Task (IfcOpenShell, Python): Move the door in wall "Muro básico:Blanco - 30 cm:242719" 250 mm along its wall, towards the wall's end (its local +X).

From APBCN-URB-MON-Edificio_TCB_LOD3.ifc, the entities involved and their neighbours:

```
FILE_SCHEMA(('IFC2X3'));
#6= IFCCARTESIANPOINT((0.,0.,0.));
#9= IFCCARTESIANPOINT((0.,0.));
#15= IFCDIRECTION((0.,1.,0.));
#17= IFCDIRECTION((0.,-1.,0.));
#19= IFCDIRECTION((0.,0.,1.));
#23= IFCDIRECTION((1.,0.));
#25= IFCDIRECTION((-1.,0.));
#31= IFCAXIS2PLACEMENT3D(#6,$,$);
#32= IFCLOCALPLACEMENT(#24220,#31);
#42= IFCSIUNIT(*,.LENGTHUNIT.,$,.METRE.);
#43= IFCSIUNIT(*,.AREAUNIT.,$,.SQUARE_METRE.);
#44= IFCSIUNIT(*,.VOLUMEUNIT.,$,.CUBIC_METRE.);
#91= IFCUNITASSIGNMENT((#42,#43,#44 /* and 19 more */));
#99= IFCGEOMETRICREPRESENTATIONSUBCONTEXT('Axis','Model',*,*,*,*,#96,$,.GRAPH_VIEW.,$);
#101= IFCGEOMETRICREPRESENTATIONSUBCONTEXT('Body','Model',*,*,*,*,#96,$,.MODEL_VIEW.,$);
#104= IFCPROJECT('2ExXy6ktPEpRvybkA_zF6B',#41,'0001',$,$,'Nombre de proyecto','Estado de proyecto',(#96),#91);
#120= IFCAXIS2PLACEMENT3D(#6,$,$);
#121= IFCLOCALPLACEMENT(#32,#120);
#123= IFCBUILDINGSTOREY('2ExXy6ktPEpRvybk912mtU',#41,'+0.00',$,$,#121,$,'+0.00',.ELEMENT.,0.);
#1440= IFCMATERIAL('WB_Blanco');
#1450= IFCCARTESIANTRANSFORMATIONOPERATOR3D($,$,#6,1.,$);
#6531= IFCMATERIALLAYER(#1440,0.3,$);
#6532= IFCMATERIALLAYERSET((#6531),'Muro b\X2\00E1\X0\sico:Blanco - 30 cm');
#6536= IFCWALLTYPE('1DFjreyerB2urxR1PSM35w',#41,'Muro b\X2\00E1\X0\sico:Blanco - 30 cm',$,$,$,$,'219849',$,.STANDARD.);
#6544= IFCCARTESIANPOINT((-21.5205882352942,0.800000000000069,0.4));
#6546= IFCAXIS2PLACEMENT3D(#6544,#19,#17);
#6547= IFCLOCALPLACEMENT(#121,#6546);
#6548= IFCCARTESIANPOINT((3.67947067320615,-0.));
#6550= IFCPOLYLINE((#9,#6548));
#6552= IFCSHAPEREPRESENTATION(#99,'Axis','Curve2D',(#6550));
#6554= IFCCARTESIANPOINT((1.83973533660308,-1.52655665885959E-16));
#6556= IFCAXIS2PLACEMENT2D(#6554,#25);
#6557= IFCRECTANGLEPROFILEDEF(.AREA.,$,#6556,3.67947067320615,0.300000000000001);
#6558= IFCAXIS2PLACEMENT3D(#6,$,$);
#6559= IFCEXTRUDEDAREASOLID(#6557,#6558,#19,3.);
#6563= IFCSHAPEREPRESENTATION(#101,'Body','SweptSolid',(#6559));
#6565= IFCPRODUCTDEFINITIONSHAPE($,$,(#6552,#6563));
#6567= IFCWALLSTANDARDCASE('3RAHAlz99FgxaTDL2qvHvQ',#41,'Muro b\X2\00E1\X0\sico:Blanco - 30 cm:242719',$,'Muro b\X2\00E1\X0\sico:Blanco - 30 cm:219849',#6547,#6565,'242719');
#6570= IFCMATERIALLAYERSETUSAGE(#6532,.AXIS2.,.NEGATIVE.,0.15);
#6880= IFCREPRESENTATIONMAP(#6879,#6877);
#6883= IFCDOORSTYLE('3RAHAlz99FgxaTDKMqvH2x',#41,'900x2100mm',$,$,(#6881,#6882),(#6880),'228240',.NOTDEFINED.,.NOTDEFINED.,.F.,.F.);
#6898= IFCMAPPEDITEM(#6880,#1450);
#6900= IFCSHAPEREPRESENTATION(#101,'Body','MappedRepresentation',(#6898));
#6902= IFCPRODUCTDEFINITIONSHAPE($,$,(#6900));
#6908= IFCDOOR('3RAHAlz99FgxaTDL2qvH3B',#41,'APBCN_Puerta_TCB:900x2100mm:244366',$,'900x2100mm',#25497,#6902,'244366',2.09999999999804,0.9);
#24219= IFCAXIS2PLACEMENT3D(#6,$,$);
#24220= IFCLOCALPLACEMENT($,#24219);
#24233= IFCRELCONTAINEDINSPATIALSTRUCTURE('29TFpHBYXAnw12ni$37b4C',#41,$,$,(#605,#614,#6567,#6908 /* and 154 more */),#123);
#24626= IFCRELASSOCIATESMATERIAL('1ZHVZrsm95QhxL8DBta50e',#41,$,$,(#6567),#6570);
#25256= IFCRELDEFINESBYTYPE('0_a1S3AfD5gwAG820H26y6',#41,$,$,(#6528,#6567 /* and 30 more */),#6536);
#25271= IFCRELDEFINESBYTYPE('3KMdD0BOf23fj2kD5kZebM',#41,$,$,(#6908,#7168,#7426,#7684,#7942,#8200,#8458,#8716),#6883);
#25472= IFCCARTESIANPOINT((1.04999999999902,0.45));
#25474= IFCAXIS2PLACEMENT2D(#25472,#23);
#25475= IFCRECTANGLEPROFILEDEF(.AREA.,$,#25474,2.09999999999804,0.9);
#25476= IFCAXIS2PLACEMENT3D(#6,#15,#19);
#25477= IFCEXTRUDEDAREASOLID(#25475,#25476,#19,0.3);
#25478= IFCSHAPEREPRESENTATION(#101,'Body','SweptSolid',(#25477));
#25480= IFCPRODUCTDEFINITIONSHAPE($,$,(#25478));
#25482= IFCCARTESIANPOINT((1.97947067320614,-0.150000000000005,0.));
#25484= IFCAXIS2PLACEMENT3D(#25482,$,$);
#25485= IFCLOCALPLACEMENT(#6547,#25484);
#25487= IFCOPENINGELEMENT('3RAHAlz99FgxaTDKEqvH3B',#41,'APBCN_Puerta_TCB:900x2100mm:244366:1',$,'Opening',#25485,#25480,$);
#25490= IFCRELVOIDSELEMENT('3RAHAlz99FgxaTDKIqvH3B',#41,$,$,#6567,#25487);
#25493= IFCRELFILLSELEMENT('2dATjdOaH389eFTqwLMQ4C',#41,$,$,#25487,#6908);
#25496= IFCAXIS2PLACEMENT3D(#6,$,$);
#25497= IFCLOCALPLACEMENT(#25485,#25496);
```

```python
import ifcopenshell
import ifcopenshell.api.geometry
import ifcopenshell.util.placement
import ifcopenshell.util.unit

model = ifcopenshell.open("APBCN-URB-MON-Edificio_TCB_LOD3.ifc")
unit_scale = ifcopenshell.util.unit.calculate_unit_scale(model)

door = model.by_guid("3RAHAlz99FgxaTDL2qvH3B")
opening = door.FillsVoids[0].RelatingOpeningElement
wall = opening.VoidsElements[0].RelatingBuildingElement

wall_matrix = ifcopenshell.util.placement.get_local_placement(wall.ObjectPlacement)
shift = wall_matrix[:3, 0] * 0.25 / unit_scale
before = ifcopenshell.util.placement.get_local_placement(door.ObjectPlacement)[:3, 3].copy()

# The door is placed relative to its opening, so it follows when the opening moves.
matrix = ifcopenshell.util.placement.get_local_placement(opening.ObjectPlacement)
matrix[:3, 3] += shift
ifcopenshell.api.geometry.edit_object_placement(
    model, product=opening, matrix=matrix, is_si=False, should_transform_children=True
)

after = ifcopenshell.util.placement.get_local_placement(door.ObjectPlacement)[:3, 3]
print("door moved by", (after - before).round(3) + 0.0)

model.write("APBCN-URB-MON-Edificio_TCB_LOD3_edited.ifc")
```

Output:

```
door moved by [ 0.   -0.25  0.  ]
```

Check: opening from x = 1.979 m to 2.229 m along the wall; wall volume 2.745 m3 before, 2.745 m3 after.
